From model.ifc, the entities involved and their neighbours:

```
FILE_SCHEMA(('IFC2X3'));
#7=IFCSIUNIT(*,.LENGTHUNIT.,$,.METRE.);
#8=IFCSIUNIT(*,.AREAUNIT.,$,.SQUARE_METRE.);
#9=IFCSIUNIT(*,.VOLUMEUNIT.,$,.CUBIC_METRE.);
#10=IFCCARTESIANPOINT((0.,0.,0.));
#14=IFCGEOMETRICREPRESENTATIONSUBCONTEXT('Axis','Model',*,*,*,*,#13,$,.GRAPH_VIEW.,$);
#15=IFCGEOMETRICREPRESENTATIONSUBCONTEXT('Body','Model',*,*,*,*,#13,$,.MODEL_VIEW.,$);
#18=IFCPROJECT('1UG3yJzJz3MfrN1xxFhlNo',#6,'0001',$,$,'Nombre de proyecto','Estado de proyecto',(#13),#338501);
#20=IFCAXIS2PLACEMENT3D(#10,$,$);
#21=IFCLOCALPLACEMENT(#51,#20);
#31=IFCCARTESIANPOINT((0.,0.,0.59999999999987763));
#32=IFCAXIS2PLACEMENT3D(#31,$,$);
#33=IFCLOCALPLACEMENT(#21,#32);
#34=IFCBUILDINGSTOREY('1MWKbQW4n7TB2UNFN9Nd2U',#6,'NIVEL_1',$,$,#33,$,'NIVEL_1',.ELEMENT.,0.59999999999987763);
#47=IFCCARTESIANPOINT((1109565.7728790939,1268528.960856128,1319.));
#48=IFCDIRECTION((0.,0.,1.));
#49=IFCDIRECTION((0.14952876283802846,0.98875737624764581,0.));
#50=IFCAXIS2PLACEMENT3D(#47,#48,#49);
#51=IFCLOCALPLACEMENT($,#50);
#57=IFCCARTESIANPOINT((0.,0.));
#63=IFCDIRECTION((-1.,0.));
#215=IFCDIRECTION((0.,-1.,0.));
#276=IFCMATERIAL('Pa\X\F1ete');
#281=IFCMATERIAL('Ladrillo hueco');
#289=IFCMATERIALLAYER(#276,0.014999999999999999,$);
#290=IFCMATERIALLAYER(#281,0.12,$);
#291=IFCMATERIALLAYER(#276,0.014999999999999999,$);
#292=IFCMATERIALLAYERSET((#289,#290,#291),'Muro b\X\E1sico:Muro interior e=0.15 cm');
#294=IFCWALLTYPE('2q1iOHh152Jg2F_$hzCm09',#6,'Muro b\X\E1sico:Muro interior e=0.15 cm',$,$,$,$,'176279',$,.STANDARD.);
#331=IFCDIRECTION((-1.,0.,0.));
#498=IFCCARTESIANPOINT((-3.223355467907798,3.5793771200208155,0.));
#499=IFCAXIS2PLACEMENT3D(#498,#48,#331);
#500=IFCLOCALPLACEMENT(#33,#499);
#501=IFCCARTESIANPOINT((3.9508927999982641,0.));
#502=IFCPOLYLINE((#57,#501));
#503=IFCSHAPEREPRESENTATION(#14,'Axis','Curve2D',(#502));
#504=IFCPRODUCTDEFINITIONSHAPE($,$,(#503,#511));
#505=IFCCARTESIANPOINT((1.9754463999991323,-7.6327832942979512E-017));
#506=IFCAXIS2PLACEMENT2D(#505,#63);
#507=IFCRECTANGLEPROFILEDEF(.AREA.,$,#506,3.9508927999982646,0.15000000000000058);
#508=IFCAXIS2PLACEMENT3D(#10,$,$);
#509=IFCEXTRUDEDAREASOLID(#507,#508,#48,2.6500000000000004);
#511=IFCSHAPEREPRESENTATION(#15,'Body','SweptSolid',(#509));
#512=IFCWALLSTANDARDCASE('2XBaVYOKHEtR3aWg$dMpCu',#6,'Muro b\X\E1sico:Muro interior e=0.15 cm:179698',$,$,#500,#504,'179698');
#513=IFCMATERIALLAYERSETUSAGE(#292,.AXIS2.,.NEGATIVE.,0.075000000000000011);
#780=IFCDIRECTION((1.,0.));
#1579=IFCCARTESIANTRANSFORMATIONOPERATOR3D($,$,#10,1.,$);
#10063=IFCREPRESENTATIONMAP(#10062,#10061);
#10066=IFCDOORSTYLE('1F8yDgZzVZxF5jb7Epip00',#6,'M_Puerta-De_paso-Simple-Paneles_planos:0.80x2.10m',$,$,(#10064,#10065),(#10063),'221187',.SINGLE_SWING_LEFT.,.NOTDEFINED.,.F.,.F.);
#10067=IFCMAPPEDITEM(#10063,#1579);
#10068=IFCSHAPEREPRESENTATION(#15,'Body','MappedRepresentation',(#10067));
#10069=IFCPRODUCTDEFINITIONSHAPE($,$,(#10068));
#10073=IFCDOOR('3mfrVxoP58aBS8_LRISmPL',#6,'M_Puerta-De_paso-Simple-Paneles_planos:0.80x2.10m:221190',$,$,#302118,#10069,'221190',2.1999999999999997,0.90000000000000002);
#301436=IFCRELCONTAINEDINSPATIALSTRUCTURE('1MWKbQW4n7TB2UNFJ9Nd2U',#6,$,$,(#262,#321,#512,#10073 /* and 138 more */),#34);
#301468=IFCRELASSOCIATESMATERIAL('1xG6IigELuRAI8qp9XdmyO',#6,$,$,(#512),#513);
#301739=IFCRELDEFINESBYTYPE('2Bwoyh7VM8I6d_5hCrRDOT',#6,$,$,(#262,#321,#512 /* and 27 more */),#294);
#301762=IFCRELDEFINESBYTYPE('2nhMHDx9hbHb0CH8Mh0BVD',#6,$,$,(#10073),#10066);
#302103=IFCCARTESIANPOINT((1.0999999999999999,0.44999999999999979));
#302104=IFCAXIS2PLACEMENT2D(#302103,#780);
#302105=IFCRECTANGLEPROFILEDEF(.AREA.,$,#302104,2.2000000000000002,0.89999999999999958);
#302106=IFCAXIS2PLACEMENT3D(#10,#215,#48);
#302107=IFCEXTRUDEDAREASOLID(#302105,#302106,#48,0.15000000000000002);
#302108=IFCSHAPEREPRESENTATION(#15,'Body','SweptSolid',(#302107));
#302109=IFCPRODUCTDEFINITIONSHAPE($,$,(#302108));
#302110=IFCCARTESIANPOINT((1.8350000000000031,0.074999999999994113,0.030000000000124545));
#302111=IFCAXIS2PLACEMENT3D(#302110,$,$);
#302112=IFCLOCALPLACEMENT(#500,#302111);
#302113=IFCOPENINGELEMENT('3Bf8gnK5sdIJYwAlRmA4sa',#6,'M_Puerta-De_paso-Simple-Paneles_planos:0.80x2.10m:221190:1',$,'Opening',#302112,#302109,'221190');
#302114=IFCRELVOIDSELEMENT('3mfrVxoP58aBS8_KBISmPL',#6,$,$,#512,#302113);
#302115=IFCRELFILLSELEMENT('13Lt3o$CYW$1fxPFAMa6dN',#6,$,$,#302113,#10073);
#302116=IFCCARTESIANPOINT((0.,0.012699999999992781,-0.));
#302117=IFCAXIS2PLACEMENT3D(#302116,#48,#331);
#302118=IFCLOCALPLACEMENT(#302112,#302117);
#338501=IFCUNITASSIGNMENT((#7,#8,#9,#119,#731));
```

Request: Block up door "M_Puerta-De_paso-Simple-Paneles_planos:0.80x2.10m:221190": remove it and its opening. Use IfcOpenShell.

```python
import ifcopenshell
import ifcopenshell.api.feature
import ifcopenshell.api.root
import ifcopenshell.geom
import ifcopenshell.util.shape

model = ifcopenshell.open("model.ifc")
settings = ifcopenshell.geom.settings()


def volume(element):
    """Net volume in cubic metres, openings subtracted."""
    shape = ifcopenshell.geom.create_shape(settings, element)
    return ifcopenshell.util.shape.get_volume(shape.geometry)


door = model.by_guid("3mfrVxoP58aBS8_LRISmPL")
opening = door.FillsVoids[0].RelatingOpeningElement
wall = opening.VoidsElements[0].RelatingBuildingElement
before = volume(wall)

ifcopenshell.api.root.remove_product(model, product=door)
ifcopenshell.api.feature.remove_feature(model, feature=opening)

after = volume(wall)

print(f"wall volume {before:.3f} -> {after:.3f} m3")

model.write("model_updated.ifc")
```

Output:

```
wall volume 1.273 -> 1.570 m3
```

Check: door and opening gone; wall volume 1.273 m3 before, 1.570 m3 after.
